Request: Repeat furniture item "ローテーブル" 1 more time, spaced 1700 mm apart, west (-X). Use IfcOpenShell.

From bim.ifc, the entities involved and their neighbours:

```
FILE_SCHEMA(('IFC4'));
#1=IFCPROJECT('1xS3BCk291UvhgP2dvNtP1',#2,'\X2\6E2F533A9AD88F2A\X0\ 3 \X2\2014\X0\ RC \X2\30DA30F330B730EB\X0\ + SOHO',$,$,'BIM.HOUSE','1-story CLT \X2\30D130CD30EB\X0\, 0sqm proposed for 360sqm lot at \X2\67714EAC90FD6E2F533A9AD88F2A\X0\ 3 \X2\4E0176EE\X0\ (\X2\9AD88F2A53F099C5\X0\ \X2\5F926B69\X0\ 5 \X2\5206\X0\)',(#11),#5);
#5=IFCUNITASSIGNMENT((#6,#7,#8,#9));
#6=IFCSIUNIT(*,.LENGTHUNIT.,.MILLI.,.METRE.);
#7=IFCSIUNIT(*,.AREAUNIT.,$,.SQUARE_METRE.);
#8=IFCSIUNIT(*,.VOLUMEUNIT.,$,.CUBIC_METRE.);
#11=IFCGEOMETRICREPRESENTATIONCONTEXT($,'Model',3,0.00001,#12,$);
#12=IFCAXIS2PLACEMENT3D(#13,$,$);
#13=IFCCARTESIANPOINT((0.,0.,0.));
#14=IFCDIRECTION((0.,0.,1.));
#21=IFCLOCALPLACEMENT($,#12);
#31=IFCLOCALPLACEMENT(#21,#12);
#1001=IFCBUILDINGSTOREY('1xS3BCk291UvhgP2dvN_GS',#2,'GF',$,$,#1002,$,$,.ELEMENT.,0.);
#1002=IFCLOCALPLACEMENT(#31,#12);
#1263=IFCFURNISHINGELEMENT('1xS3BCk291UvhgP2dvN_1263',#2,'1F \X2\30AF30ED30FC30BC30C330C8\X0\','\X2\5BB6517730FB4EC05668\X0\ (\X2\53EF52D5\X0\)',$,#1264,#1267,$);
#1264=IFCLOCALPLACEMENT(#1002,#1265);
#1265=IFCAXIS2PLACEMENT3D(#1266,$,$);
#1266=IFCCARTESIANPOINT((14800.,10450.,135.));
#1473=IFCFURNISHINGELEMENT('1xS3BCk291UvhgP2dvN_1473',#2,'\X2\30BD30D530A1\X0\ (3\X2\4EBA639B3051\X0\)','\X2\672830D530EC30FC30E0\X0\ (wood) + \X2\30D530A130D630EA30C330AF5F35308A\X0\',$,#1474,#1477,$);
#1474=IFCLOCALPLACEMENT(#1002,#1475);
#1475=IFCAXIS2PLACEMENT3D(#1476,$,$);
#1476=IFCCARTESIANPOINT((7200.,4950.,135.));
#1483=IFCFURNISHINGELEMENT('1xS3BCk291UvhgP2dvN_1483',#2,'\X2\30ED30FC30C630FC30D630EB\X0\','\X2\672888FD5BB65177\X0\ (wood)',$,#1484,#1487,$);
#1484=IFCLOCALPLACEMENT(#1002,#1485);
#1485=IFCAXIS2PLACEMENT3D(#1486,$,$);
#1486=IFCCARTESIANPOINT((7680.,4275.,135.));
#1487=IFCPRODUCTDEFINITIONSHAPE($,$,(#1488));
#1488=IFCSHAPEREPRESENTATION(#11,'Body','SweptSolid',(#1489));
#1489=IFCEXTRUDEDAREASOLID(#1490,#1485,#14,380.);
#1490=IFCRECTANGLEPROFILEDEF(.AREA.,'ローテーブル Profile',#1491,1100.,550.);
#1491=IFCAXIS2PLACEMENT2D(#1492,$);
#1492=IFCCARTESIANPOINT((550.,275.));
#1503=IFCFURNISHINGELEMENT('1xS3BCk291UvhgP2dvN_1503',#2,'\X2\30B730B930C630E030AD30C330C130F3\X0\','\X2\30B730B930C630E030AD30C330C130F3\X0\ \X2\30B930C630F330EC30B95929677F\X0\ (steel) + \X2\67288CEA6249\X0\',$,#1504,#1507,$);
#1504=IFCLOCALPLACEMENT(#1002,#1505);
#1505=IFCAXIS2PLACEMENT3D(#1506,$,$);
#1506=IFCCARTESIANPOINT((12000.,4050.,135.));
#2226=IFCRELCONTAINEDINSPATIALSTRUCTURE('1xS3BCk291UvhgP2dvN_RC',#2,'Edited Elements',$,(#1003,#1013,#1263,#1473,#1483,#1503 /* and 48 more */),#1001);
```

```python
import numpy as np
import ifcopenshell
import ifcopenshell.api.geometry
import ifcopenshell.api.root
import ifcopenshell.util.element
import ifcopenshell.util.placement
import ifcopenshell.util.unit

model = ifcopenshell.open("bim.ifc")
unit_scale = ifcopenshell.util.unit.calculate_unit_scale(model)


def reuse_history(source, copy):
    """copy_class also copies each property set's owner history, people and application; keep the originals."""
    for rel in copy.IsDefinedBy:
        if rel.is_a("IfcRelDefinesByProperties") and (history := rel.RelatingPropertyDefinition.OwnerHistory):
            rel.RelatingPropertyDefinition.OwnerHistory = source.OwnerHistory
            ifcopenshell.util.element.remove_deep2(model, history)


source = model.by_id(1483)
base = ifcopenshell.util.placement.get_local_placement(source.ObjectPlacement)
step = np.array([-1.0, 0.0, 0.0]) * 1.7 / unit_scale

for i in range(1, 2):
    copy = ifcopenshell.api.root.copy_class(model, product=source)
    copy.Representation = ifcopenshell.util.element.copy_deep(
        model, source.Representation, exclude=["IfcGeometricRepresentationContext", "IfcRepresentationMap"]
    )
    reuse_history(source, copy)
    matrix = base.copy()
    matrix[:3, 3] += i * step
    print("added at", matrix[:3, 3].round(3) + 0.0)
    ifcopenshell.api.geometry.edit_object_placement(model, product=copy, matrix=matrix, is_si=False)

model.write("bim_rev.ifc")
```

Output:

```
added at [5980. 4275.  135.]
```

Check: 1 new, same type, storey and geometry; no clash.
